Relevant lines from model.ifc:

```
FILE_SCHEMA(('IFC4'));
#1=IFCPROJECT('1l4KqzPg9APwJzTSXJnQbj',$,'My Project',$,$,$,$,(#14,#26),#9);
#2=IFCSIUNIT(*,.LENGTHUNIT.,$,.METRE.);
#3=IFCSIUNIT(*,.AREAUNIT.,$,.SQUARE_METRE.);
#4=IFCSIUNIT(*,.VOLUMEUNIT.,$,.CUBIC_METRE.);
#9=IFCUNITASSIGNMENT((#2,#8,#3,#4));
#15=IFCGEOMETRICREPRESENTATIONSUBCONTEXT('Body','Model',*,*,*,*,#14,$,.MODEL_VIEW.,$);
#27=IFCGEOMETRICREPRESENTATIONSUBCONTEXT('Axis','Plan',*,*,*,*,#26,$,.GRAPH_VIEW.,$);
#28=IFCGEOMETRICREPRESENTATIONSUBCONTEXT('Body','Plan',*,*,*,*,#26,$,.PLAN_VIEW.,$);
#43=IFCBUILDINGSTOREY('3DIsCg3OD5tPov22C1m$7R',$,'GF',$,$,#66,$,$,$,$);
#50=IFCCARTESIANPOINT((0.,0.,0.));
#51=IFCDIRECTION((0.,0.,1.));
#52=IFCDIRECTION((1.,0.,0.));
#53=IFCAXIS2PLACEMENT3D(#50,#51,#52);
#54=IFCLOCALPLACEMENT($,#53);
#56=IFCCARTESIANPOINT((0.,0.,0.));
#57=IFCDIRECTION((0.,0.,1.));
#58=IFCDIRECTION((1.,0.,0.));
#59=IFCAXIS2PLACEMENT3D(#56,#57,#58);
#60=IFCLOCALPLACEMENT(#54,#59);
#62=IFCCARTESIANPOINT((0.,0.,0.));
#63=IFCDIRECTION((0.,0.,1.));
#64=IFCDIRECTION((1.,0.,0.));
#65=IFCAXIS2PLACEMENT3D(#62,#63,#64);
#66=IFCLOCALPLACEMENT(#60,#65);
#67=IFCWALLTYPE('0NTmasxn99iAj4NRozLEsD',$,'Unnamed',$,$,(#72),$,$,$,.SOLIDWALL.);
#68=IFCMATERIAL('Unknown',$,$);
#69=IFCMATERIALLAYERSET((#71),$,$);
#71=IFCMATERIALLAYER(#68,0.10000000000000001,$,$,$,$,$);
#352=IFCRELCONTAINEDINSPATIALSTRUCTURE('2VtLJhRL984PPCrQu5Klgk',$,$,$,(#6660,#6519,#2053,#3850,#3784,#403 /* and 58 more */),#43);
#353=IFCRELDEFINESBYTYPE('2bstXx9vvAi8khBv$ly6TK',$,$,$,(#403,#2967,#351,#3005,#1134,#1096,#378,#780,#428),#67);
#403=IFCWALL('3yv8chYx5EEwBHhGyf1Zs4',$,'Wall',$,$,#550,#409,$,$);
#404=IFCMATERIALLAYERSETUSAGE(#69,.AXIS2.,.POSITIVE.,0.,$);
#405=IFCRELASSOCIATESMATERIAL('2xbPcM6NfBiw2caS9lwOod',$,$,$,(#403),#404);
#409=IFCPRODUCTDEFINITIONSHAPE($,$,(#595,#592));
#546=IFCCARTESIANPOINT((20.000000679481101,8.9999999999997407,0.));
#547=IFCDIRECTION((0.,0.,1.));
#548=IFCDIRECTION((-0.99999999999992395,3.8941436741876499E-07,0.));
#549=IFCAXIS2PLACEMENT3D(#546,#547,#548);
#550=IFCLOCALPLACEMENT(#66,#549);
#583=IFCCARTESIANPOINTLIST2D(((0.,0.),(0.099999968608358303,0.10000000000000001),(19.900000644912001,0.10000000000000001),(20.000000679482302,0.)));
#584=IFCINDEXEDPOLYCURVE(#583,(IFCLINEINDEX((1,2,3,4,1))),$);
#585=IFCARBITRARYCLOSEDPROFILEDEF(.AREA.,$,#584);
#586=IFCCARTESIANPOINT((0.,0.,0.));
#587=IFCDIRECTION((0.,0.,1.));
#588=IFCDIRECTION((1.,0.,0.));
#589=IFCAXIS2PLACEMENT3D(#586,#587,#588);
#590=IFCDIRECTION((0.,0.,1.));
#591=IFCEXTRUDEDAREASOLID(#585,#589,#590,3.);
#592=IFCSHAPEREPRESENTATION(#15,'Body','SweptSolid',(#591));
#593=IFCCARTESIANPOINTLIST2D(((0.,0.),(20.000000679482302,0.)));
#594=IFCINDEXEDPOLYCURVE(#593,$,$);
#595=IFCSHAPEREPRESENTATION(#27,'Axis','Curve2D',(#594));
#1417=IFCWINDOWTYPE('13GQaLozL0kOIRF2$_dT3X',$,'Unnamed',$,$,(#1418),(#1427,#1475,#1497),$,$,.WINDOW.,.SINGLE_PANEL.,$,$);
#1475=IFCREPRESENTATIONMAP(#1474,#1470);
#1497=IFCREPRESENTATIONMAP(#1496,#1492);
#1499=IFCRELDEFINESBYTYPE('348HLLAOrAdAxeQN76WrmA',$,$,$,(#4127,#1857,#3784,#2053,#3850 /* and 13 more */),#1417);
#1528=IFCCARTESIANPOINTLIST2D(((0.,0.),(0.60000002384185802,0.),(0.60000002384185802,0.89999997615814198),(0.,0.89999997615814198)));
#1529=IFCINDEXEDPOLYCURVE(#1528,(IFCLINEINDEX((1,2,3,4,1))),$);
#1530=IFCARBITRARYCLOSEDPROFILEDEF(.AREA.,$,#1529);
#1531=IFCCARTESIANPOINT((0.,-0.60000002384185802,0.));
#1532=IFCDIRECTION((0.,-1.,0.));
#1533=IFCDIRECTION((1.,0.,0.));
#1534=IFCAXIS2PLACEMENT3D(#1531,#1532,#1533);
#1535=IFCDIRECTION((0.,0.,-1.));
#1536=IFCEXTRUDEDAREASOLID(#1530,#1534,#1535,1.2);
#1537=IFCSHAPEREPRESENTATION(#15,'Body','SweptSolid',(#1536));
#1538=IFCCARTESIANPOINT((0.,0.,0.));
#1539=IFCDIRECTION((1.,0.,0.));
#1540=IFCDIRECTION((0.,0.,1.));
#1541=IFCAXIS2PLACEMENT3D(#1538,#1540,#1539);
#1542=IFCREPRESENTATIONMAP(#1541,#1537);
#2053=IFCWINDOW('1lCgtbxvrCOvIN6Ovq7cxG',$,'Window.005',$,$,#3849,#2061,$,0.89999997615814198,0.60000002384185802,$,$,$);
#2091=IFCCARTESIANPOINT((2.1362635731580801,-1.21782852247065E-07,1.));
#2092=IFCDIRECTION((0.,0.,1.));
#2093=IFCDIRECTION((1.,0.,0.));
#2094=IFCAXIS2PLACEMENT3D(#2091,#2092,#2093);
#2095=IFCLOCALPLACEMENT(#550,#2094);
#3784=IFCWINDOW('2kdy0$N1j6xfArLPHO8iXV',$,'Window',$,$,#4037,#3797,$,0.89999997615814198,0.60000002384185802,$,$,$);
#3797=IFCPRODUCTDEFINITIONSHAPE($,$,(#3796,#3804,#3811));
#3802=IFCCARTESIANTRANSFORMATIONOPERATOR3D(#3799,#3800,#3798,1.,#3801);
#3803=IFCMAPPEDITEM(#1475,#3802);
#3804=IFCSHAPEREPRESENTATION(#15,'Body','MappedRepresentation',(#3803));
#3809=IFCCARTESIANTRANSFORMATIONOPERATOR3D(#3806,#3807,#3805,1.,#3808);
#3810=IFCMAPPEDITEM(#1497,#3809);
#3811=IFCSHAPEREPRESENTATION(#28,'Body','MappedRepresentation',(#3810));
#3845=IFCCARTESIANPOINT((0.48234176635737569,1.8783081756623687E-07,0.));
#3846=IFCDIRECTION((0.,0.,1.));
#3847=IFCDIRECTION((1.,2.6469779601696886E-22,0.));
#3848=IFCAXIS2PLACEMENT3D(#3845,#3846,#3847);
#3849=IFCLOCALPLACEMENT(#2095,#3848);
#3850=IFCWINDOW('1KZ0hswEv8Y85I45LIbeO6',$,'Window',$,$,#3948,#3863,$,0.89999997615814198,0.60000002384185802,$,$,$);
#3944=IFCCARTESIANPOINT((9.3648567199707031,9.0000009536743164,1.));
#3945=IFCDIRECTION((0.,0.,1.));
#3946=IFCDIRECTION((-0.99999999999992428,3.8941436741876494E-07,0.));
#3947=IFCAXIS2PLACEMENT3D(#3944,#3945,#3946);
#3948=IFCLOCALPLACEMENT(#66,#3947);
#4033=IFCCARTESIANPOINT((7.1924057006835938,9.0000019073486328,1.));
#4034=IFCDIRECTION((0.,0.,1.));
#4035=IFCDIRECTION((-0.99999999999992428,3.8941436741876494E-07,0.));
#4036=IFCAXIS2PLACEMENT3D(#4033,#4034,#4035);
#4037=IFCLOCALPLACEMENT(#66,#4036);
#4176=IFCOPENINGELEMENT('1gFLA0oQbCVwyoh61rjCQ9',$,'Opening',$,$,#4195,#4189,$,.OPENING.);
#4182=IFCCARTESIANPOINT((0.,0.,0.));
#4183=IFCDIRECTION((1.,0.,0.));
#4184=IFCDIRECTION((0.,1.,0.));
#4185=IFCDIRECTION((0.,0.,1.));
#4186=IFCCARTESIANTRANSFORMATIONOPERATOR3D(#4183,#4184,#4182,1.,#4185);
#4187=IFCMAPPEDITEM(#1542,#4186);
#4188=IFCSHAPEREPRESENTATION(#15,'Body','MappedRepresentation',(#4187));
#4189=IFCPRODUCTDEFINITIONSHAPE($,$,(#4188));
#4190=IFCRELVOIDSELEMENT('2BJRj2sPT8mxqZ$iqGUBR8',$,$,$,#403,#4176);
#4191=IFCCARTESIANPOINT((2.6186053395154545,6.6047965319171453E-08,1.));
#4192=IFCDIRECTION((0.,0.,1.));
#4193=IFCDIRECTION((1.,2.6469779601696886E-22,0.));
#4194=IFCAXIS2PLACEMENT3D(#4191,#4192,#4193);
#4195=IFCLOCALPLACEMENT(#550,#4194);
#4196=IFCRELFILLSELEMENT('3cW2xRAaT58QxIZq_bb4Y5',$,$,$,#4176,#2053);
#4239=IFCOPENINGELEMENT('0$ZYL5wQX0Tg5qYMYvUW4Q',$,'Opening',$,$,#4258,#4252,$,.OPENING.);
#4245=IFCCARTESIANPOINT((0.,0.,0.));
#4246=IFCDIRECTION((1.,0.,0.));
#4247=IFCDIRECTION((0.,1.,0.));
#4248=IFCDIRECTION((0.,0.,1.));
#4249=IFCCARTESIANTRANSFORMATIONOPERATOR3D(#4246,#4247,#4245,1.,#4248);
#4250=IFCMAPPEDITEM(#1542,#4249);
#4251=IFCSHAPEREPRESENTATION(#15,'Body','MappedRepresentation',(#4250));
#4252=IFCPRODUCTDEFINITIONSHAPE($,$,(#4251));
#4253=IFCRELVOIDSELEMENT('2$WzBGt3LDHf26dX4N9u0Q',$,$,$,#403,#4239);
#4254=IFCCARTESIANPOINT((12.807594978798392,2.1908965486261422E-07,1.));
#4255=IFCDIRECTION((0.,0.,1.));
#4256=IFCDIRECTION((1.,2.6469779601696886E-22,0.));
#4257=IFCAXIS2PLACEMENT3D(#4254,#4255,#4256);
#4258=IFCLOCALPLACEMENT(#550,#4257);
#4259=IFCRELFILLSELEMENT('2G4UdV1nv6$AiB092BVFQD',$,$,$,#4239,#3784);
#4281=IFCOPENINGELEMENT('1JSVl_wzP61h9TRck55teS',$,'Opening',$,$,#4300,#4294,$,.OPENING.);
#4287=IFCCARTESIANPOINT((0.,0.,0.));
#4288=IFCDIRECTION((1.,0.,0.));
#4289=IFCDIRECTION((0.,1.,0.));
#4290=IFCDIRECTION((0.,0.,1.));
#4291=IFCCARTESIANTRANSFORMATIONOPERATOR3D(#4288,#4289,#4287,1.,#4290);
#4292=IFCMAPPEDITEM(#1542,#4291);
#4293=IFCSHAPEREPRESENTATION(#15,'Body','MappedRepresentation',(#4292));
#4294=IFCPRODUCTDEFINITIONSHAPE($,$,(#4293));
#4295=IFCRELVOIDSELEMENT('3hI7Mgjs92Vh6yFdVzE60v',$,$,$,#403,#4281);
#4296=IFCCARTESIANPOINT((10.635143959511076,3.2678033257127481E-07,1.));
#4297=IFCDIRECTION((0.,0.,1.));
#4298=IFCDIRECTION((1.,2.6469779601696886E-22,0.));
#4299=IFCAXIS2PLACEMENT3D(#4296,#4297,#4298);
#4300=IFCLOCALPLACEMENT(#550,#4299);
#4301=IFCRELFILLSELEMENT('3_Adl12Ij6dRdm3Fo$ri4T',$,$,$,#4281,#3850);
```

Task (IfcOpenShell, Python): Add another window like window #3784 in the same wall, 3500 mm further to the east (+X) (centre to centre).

```python
import ifcopenshell
import ifcopenshell.api.feature
import ifcopenshell.api.geometry
import ifcopenshell.api.root
import ifcopenshell.geom
import ifcopenshell.util.element
import ifcopenshell.util.placement
import ifcopenshell.util.shape

model = ifcopenshell.open("model.ifc")
settings = ifcopenshell.geom.settings()


def volume(element):
    """Net volume in cubic metres, openings subtracted."""
    shape = ifcopenshell.geom.create_shape(settings, element)
    return ifcopenshell.util.shape.get_volume(shape.geometry)


window = model.by_guid("2kdy0$N1j6xfArLPHO8iXV")
opening = window.FillsVoids[0].RelatingOpeningElement
wall = opening.VoidsElements[0].RelatingBuildingElement
before = volume(wall)
shift = ifcopenshell.util.placement.get_local_placement(wall.ObjectPlacement)[:3, 0] * -3.5

# copy_class copies the void relationship, type, container and properties, but no geometry.
new_opening = ifcopenshell.api.root.copy_class(model, product=opening)
new_opening.Representation = ifcopenshell.util.element.copy_deep(
    model, opening.Representation, exclude=["IfcGeometricRepresentationContext", "IfcRepresentationMap"]
)
new_window = ifcopenshell.api.root.copy_class(model, product=window)
new_window.Representation = ifcopenshell.util.element.copy_deep(
    model, window.Representation, exclude=["IfcGeometricRepresentationContext", "IfcRepresentationMap"]
)
ifcopenshell.api.feature.add_filling(model, opening=new_opening, element=new_window)

for old, new in ((opening, new_opening), (window, new_window)):
    matrix = ifcopenshell.util.placement.get_local_placement(old.ObjectPlacement)
    matrix[:3, 3] += shift
    ifcopenshell.api.geometry.edit_object_placement(model, product=new, matrix=matrix, is_si=False)

after = volume(wall)

print(f"wall volume {before:.3f} -> {after:.3f} m3")

model.write("model_v2.ifc")
```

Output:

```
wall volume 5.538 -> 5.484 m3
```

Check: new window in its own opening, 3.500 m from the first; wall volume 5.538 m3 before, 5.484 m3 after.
